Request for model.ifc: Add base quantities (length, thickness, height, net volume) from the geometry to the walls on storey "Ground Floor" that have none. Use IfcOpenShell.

First a look at what the model holds.

```python
import ifcopenshell
import ifcopenshell.util.element
import ifcopenshell.util.unit

model = ifcopenshell.open("model.ifc")
print(model.schema)
for unit_type in ("LENGTHUNIT", "AREAUNIT", "VOLUMEUNIT"):
    print(unit_type, ifcopenshell.util.unit.calculate_unit_scale(model, unit_type))
storey = next(s for s in model.by_type("IfcBuildingStorey") if s.Name == "Ground Floor")
walls = [e for e in ifcopenshell.util.element.get_decomposition(storey) if e.is_a("IfcWall")]
for e in sorted(walls, key=lambda e: e.id()):
    print(e.id(), e.is_a(), e.Name, list(ifcopenshell.util.element.get_psets(e, qtos_only=True)), sep=" | ")
```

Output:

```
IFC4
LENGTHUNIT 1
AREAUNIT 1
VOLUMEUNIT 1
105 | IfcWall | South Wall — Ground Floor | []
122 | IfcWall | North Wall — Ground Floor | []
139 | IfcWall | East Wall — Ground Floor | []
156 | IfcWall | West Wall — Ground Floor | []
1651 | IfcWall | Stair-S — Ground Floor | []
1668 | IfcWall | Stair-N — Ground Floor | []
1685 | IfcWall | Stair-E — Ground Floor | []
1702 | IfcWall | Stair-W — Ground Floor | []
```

```python
import ifcopenshell
import ifcopenshell.api.pset
import ifcopenshell.geom
import ifcopenshell.util.element
import ifcopenshell.util.shape
import ifcopenshell.util.unit

model = ifcopenshell.open("model.ifc")
unit_scale = ifcopenshell.util.unit.calculate_unit_scale(model)
volume_scale = ifcopenshell.util.unit.calculate_unit_scale(model, "VOLUMEUNIT")
settings = ifcopenshell.geom.settings()

storey = next(s for s in model.by_type("IfcBuildingStorey") if s.Name == "Ground Floor")
walls = [e for e in ifcopenshell.util.element.get_decomposition(storey) if e.is_a("IfcWall")]

for e in sorted(walls, key=lambda e: e.id()):
    if ifcopenshell.util.element.get_psets(e, qtos_only=True, should_inherit=False):
        continue
    # Geometry comes back in metres, in the element's own axes.
    shape = ifcopenshell.geom.create_shape(settings, e)
    values = {
        "Length": ifcopenshell.util.shape.get_x(shape.geometry) / unit_scale,
        "Width": ifcopenshell.util.shape.get_y(shape.geometry) / unit_scale,
        "Height": ifcopenshell.util.shape.get_z(shape.geometry) / unit_scale,
        "NetVolume": ifcopenshell.util.shape.get_volume(shape.geometry) / volume_scale,
    }
    qto = ifcopenshell.api.pset.add_qto(model, product=e, name="Qto_WallBaseQuantities")
    ifcopenshell.api.pset.edit_qto(model, qto=qto, properties=values)
    print(e.id(), {k: round(v, 3) for k, v in values.items()})

model.write("model_updated.ifc")
```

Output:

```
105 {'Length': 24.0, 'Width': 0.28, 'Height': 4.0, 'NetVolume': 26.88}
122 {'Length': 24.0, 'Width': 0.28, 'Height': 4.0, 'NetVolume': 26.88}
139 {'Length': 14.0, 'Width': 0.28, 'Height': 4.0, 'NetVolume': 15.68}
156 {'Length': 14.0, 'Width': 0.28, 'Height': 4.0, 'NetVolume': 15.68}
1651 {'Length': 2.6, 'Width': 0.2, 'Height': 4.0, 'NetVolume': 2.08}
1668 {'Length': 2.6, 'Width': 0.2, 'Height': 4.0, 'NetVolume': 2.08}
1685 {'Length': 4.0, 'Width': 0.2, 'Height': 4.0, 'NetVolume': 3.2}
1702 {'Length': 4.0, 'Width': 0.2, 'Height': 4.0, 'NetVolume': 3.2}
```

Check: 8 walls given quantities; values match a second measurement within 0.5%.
